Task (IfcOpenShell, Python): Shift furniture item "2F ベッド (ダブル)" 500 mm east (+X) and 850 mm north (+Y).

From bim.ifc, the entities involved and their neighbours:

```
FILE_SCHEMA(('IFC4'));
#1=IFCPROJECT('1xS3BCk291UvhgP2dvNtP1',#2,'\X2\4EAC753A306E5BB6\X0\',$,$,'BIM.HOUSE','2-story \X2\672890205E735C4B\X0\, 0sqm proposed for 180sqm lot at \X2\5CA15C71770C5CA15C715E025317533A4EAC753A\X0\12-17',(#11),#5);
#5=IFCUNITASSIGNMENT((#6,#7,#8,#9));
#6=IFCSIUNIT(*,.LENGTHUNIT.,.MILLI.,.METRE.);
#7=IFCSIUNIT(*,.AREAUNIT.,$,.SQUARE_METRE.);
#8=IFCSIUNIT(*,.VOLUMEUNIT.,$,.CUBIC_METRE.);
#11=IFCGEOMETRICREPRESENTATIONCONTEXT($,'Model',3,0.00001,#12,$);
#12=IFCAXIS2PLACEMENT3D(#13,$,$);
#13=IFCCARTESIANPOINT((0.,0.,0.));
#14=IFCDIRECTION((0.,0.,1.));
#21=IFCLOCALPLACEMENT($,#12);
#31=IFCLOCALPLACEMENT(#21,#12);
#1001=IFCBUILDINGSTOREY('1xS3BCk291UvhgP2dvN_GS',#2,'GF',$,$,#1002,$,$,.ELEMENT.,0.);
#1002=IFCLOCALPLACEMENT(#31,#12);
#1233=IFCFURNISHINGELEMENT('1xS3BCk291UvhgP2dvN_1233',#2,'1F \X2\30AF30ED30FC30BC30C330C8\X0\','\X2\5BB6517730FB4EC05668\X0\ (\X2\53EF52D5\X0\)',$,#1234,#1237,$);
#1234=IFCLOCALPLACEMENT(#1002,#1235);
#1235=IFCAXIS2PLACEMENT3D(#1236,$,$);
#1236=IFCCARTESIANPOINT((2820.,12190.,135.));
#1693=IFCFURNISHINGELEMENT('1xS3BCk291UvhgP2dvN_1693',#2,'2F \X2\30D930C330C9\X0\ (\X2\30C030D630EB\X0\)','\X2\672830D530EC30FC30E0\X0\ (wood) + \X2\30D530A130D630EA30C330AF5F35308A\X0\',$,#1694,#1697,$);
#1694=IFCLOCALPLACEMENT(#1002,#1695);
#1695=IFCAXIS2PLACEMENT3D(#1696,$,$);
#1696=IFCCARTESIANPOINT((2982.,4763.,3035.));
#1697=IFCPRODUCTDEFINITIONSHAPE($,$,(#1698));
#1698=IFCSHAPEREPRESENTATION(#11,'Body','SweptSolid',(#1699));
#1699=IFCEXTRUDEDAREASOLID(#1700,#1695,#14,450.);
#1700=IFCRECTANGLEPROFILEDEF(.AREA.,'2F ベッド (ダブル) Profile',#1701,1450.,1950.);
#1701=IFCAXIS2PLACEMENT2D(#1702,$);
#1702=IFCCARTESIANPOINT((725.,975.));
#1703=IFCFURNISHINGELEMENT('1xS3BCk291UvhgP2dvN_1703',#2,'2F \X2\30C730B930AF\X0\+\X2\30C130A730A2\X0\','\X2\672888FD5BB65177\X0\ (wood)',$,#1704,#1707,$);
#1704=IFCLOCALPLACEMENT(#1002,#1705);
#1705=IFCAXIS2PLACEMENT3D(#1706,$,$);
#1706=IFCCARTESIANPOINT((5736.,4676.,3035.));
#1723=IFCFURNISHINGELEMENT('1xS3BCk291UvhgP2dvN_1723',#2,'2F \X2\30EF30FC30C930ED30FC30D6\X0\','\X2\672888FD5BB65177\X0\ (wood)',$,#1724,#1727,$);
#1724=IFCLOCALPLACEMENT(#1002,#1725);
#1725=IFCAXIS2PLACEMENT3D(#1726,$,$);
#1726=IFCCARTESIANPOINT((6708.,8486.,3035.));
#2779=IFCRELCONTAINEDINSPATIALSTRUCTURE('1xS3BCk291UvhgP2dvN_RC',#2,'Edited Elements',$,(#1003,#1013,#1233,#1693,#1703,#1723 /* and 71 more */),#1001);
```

```python
import ifcopenshell
import ifcopenshell.api.geometry
import ifcopenshell.util.placement

model = ifcopenshell.open("bim.ifc")

item = model.by_guid("1xS3BCk291UvhgP2dvN_1693")
matrix = ifcopenshell.util.placement.get_local_placement(item.ObjectPlacement)
matrix[0, 3] += 500.0
matrix[1, 3] += 850.0
ifcopenshell.api.geometry.edit_object_placement(model, product=item, matrix=matrix, is_si=False)

print(ifcopenshell.util.placement.get_local_placement(item.ObjectPlacement).round(3) + 0.0)

model.write("bim_updated.ifc")
```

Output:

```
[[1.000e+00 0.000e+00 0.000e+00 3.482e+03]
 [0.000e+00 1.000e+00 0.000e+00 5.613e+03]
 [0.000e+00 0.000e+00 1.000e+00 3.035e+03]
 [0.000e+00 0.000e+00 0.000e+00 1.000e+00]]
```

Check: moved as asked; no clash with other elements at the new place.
